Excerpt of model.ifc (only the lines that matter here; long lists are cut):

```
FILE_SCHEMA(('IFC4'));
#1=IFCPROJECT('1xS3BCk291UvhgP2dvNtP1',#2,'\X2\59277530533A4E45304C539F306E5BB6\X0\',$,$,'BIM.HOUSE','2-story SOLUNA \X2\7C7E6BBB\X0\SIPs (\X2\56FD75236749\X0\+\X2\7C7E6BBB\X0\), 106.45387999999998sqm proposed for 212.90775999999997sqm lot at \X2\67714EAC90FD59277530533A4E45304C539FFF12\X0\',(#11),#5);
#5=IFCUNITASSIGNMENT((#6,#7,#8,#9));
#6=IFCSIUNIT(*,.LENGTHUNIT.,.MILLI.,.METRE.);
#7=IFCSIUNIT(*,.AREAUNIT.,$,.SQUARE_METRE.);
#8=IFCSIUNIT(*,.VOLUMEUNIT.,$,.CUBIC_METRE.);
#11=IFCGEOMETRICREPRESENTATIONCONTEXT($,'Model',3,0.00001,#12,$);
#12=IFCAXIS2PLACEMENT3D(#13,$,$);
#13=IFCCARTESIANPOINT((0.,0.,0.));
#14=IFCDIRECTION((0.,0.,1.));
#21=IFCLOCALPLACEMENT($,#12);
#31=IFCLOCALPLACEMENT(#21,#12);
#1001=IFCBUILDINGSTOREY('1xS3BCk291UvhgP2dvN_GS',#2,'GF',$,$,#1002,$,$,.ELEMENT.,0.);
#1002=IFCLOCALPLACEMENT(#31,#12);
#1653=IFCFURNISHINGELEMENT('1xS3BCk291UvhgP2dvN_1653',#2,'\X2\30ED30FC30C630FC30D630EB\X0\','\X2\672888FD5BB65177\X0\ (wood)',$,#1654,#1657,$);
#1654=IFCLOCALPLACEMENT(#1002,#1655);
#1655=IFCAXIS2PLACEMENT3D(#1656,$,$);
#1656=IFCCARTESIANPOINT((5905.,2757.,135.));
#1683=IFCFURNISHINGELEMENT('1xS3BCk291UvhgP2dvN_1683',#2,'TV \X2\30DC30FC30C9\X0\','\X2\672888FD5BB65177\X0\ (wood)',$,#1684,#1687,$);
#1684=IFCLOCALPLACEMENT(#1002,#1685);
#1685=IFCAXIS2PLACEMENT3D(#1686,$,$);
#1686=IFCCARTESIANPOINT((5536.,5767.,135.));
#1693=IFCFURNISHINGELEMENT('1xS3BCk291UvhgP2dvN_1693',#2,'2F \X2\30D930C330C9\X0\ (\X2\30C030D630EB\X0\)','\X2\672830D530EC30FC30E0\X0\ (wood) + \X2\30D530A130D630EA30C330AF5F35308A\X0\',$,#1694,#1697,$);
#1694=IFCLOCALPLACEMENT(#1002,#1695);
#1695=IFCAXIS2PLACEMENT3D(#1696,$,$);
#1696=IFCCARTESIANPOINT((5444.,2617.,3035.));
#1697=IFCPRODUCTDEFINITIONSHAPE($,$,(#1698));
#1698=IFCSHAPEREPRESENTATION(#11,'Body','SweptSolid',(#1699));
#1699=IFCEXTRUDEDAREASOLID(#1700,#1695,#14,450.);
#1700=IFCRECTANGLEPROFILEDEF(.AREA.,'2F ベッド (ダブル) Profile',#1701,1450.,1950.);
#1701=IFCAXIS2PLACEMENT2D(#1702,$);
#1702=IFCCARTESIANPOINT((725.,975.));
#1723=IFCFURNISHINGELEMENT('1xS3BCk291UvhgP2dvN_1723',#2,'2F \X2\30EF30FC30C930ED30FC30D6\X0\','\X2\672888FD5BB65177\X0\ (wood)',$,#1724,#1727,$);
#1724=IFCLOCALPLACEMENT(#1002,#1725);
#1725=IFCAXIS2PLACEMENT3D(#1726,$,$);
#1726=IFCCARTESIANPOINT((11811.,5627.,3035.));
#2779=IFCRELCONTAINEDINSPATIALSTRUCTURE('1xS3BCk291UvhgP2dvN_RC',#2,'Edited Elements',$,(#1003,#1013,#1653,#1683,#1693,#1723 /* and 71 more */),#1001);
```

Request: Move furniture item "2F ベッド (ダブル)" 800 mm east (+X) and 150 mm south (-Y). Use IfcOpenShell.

```python
import ifcopenshell
import ifcopenshell.api.geometry
import ifcopenshell.util.placement

model = ifcopenshell.open("model.ifc")

item = model.by_guid("1xS3BCk291UvhgP2dvN_1693")
matrix = ifcopenshell.util.placement.get_local_placement(item.ObjectPlacement)
matrix[0, 3] += 800.0
matrix[1, 3] -= 150.0
ifcopenshell.api.geometry.edit_object_placement(model, product=item, matrix=matrix, is_si=False)

print(ifcopenshell.util.placement.get_local_placement(item.ObjectPlacement).round(3) + 0.0)

model.write("model_updated.ifc")
```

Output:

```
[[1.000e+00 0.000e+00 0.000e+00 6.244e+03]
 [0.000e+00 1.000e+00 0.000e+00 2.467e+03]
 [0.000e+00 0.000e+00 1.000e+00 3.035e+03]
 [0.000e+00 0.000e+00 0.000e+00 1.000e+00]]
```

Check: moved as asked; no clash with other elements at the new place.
